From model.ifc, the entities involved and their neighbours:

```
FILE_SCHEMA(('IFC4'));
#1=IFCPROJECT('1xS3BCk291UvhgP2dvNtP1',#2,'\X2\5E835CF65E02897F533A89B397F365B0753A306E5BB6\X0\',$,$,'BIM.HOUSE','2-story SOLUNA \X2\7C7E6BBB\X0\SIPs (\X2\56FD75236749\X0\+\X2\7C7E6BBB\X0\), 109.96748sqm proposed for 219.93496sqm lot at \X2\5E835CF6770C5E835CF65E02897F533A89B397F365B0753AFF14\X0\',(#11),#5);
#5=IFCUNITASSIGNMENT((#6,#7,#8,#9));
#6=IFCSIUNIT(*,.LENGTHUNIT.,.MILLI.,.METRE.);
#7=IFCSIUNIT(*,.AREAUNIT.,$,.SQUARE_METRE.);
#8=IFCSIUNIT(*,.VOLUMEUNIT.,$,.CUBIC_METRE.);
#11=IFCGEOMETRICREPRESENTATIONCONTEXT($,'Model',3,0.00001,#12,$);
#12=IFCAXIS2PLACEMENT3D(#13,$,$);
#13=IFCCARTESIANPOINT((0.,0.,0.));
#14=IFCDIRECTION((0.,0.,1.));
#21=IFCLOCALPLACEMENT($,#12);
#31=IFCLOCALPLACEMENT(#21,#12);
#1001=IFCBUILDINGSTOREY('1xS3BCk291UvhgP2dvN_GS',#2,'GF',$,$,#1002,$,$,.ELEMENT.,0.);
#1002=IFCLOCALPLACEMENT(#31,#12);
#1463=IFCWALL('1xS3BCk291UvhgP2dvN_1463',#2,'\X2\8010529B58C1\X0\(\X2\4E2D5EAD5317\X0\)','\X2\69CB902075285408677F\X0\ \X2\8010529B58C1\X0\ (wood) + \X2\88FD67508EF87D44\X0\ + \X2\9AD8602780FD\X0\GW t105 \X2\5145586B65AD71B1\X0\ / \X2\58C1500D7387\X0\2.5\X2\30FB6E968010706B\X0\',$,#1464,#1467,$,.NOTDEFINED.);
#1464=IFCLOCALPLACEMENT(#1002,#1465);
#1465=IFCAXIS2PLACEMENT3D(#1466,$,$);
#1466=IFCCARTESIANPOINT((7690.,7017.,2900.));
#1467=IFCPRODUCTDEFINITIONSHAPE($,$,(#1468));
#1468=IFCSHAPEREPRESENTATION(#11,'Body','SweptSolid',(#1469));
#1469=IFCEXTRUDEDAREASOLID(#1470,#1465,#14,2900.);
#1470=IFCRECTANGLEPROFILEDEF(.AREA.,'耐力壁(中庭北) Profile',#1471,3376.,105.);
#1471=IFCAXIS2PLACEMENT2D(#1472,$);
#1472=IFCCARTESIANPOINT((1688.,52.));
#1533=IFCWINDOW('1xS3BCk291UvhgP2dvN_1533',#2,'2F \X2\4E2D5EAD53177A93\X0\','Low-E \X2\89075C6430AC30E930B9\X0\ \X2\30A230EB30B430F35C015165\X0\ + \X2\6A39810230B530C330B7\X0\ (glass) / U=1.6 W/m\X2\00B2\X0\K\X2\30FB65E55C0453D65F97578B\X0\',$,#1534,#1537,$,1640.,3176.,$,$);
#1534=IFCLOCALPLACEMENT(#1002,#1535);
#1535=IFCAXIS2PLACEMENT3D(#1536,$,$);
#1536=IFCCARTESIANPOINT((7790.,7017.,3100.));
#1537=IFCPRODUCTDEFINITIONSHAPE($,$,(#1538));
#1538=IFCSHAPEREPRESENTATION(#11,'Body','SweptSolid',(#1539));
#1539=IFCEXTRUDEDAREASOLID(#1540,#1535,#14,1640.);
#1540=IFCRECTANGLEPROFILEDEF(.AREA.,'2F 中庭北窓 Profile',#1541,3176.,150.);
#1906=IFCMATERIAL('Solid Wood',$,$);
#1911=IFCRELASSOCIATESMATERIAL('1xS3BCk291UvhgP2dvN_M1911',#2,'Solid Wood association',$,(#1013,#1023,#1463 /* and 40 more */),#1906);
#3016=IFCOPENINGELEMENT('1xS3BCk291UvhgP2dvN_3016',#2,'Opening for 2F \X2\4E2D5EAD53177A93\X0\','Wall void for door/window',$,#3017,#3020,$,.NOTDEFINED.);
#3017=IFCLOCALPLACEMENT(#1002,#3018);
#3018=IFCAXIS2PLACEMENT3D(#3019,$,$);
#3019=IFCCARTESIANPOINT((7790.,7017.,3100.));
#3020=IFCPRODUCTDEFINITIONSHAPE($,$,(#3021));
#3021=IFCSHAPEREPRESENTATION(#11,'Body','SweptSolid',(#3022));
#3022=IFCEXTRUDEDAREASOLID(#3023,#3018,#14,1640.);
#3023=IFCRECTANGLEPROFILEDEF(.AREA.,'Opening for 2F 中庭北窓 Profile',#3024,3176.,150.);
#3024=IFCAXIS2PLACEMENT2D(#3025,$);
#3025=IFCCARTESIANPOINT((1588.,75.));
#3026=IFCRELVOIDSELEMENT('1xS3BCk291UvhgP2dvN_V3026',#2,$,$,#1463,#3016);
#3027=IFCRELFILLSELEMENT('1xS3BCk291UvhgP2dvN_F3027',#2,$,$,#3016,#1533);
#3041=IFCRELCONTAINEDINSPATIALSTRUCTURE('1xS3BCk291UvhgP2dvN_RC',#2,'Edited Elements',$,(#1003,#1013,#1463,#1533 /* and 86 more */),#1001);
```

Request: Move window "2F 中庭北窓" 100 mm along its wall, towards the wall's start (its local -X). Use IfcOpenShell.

```python
import ifcopenshell
import ifcopenshell.api.geometry
import ifcopenshell.util.placement
import ifcopenshell.util.unit

model = ifcopenshell.open("model.ifc")
unit_scale = ifcopenshell.util.unit.calculate_unit_scale(model)

window = model.by_guid("1xS3BCk291UvhgP2dvN_1533")
opening = window.FillsVoids[0].RelatingOpeningElement
wall = opening.VoidsElements[0].RelatingBuildingElement

wall_matrix = ifcopenshell.util.placement.get_local_placement(wall.ObjectPlacement)
shift = wall_matrix[:3, 0] * -0.1 / unit_scale
before = ifcopenshell.util.placement.get_local_placement(window.ObjectPlacement)[:3, 3].copy()

# The window is not placed relative to its opening, so move both.
for product in (opening, window):
    matrix = ifcopenshell.util.placement.get_local_placement(product.ObjectPlacement)
    matrix[:3, 3] += shift
    ifcopenshell.api.geometry.edit_object_placement(model, product=product, matrix=matrix, is_si=False)

after = ifcopenshell.util.placement.get_local_placement(window.ObjectPlacement)[:3, 3]
print("window moved by", (after - before).round(3) + 0.0)

model.write("model_rev.ifc")
```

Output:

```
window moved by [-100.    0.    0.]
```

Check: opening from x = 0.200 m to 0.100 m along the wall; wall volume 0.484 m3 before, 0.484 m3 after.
